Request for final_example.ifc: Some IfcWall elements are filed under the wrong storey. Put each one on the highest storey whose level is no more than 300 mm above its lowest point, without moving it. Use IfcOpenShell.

First a look at what the model holds.

```python
import ifcopenshell
import ifcopenshell.util.element
import ifcopenshell.util.placement

model = ifcopenshell.open("final_example.ifc")
print(model.schema)
for storey in model.by_type("IfcBuildingStorey"):
    level = ifcopenshell.util.placement.get_storey_elevation(storey)
    count = sum(e.is_a("IfcWall") for e in ifcopenshell.util.element.get_contained(storey))
    print(storey.id(), storey.Name, round(level, 3), count, sep=" | ")
```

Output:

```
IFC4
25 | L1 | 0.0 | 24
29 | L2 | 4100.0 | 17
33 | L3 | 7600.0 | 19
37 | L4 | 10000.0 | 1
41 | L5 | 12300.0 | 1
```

```python
import ifcopenshell
import ifcopenshell.api.spatial
import ifcopenshell.geom
import ifcopenshell.util.element
import ifcopenshell.util.placement
import ifcopenshell.util.shape
import ifcopenshell.util.unit

model = ifcopenshell.open("final_example.ifc")
unit_scale = ifcopenshell.util.unit.calculate_unit_scale(model)
settings = ifcopenshell.geom.settings()

levels = sorted(
    ((ifcopenshell.util.placement.get_storey_elevation(s) * unit_scale, s) for s in model.by_type("IfcBuildingStorey")),
    key=lambda pair: pair[0],
)

for e in model.by_type("IfcWall"):
    current = e.ContainedInStructure[0].RelatingStructure if e.ContainedInStructure else None
    if current is None or not current.is_a("IfcBuildingStorey"):
        continue
    shape = ifcopenshell.geom.create_shape(settings, e)
    bottom = ifcopenshell.util.shape.get_shape_bottom_elevation(shape, shape.geometry)
    below = [s for level, s in levels if level <= bottom + 0.3]
    storey = below[-1] if below else levels[0][1]
    if storey != current:
        # assign_container keeps the world position.
        ifcopenshell.api.spatial.assign_container(model, products=[e], relating_structure=storey)
        print(e.id(), current.Name, "->", storey.Name)

model.write("final_example_edited.ifc")
```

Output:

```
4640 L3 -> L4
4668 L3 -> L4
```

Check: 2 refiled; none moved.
